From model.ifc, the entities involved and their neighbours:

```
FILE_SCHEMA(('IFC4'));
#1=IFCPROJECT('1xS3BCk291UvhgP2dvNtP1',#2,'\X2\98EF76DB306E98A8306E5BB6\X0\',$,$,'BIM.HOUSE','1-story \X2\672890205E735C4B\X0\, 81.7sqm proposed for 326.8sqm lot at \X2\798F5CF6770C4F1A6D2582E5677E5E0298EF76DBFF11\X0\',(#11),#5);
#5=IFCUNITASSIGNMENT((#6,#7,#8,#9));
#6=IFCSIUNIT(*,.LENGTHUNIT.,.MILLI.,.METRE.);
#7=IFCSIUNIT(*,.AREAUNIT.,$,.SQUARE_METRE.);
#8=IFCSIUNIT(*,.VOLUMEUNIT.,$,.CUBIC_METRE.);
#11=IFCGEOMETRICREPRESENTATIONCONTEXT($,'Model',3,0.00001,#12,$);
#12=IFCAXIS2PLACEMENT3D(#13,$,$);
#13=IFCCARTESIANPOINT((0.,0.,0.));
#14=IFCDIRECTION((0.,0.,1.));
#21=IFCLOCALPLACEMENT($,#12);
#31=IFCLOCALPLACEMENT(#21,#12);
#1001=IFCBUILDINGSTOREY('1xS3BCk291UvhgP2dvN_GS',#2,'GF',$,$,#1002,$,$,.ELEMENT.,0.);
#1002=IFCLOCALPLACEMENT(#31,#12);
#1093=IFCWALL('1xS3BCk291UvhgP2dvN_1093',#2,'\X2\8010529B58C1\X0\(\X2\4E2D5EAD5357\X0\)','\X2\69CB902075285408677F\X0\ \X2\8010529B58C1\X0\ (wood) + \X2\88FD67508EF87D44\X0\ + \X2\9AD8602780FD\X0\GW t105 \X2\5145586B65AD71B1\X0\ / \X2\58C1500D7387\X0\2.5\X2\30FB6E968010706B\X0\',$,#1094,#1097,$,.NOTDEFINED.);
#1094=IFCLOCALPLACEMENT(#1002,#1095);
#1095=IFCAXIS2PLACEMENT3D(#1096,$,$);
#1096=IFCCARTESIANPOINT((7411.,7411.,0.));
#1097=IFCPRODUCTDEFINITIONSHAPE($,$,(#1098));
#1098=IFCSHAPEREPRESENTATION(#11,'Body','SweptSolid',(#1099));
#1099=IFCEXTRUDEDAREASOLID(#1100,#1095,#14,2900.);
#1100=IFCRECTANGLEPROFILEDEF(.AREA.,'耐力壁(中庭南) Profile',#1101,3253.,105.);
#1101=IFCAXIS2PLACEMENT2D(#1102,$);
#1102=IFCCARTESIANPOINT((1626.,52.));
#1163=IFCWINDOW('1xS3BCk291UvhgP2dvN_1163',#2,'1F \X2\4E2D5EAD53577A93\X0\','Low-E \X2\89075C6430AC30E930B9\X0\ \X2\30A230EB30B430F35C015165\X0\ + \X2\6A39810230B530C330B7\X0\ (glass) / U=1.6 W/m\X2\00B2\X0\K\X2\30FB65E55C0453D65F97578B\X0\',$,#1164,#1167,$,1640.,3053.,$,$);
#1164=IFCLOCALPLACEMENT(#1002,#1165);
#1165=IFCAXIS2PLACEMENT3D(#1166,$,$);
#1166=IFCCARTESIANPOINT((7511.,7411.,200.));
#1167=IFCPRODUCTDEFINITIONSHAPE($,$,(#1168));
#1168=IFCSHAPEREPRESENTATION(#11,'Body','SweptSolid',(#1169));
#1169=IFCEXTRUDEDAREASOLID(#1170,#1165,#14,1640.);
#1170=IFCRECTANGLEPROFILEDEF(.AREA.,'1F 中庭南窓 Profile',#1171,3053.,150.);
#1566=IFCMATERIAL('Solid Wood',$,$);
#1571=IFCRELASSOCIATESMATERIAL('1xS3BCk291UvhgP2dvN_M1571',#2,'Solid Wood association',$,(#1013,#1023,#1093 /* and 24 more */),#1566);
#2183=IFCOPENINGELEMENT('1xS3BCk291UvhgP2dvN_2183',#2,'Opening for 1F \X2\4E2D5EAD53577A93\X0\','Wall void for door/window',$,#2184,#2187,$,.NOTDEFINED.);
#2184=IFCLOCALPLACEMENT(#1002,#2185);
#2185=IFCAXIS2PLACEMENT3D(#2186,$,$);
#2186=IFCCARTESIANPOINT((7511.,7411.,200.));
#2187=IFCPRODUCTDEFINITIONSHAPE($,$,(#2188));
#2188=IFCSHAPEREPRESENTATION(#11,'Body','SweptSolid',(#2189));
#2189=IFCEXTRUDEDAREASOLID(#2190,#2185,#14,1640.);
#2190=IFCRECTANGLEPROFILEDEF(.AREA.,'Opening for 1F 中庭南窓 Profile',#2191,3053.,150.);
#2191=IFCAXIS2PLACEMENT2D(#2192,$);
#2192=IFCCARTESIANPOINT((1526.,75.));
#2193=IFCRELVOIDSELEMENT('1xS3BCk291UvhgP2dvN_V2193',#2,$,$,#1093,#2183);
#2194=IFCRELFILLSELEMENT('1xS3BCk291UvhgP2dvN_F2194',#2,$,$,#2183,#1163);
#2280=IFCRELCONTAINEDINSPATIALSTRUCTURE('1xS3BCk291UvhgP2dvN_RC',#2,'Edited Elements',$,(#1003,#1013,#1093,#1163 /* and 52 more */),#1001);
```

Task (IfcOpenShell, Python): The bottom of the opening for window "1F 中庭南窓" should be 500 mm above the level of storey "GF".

```python
import numpy as np
import ifcopenshell
import ifcopenshell.api.geometry
import ifcopenshell.geom
import ifcopenshell.util.element
import ifcopenshell.util.placement
import ifcopenshell.util.shape
import ifcopenshell.util.unit

model = ifcopenshell.open("model.ifc")
unit_scale = ifcopenshell.util.unit.calculate_unit_scale(model)

window = model.by_guid("1xS3BCk291UvhgP2dvN_1163")
opening = window.FillsVoids[0].RelatingOpeningElement
storey = ifcopenshell.util.element.get_container(window, ifc_class="IfcBuildingStorey")
level = ifcopenshell.util.placement.get_local_placement(storey.ObjectPlacement)[2, 3]

# The opening's origin need not be at the sill, so measure its lowest point.
shape = ifcopenshell.geom.create_shape(ifcopenshell.geom.settings(), opening)
bottom = ifcopenshell.util.shape.get_shape_bottom_elevation(shape, shape.geometry) / unit_scale
dz = level + 0.5 / unit_scale - bottom

shift = np.array([0.0, 0.0, dz])
# The window is not placed relative to its opening, so move both.
for product in (opening, window):
    matrix = ifcopenshell.util.placement.get_local_placement(product.ObjectPlacement)
    matrix[:3, 3] += shift
    ifcopenshell.api.geometry.edit_object_placement(model, product=product, matrix=matrix, is_si=False)

print(f"moved by {dz * unit_scale:+.3f} m")

model.write("model_edited.ifc")
```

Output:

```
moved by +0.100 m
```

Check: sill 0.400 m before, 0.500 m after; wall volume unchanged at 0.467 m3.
